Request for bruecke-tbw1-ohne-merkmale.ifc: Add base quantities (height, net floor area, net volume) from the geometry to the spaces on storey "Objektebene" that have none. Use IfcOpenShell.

First a look at what the model holds.

```python
import ifcopenshell
import ifcopenshell.util.element
import ifcopenshell.util.unit

model = ifcopenshell.open("bruecke-tbw1-ohne-merkmale.ifc")
print(model.schema)
for unit_type in ("LENGTHUNIT", "AREAUNIT", "VOLUMEUNIT"):
    print(unit_type, ifcopenshell.util.unit.calculate_unit_scale(model, unit_type))
storey = next(s for s in model.by_type("IfcBuildingStorey") if s.Name == "Objektebene")
spaces = [e for e in ifcopenshell.util.element.get_decomposition(storey) if e.is_a("IfcSpace")]
for e in sorted(spaces, key=lambda e: e.id()):
    print(e.id(), e.is_a(), e.Name, list(ifcopenshell.util.element.get_psets(e, qtos_only=True)), sep=" | ")
```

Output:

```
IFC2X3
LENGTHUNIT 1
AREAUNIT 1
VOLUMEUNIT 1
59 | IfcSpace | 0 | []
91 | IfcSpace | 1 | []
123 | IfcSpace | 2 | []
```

```python
import ifcopenshell
import ifcopenshell.api.pset
import ifcopenshell.geom
import ifcopenshell.util.element
import ifcopenshell.util.shape
import ifcopenshell.util.unit

model = ifcopenshell.open("bruecke-tbw1-ohne-merkmale.ifc")
unit_scale = ifcopenshell.util.unit.calculate_unit_scale(model)
area_scale = ifcopenshell.util.unit.calculate_unit_scale(model, "AREAUNIT")
volume_scale = ifcopenshell.util.unit.calculate_unit_scale(model, "VOLUMEUNIT")
settings = ifcopenshell.geom.settings()

storey = next(s for s in model.by_type("IfcBuildingStorey") if s.Name == "Objektebene")
spaces = [e for e in ifcopenshell.util.element.get_decomposition(storey) if e.is_a("IfcSpace")]

for e in sorted(spaces, key=lambda e: e.id()):
    if ifcopenshell.util.element.get_psets(e, qtos_only=True, should_inherit=False):
        continue
    # Geometry comes back in metres, in the element's own axes.
    shape = ifcopenshell.geom.create_shape(settings, e)
    values = {
        "Height": ifcopenshell.util.shape.get_z(shape.geometry) / unit_scale,
        "NetFloorArea": ifcopenshell.util.shape.get_footprint_area(shape.geometry) / area_scale,
        "NetVolume": ifcopenshell.util.shape.get_volume(shape.geometry) / volume_scale,
    }
    qto = ifcopenshell.api.pset.add_qto(model, product=e, name="BaseQuantities")
    ifcopenshell.api.pset.edit_qto(model, qto=qto, properties=values)
    print(e.id(), {k: round(v, 3) for k, v in values.items()})

model.write("bruecke-tbw1-ohne-merkmale-out.ifc")
```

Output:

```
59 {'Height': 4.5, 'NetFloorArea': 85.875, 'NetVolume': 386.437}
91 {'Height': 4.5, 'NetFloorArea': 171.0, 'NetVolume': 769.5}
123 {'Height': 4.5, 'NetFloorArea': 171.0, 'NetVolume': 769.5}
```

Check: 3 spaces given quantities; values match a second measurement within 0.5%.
